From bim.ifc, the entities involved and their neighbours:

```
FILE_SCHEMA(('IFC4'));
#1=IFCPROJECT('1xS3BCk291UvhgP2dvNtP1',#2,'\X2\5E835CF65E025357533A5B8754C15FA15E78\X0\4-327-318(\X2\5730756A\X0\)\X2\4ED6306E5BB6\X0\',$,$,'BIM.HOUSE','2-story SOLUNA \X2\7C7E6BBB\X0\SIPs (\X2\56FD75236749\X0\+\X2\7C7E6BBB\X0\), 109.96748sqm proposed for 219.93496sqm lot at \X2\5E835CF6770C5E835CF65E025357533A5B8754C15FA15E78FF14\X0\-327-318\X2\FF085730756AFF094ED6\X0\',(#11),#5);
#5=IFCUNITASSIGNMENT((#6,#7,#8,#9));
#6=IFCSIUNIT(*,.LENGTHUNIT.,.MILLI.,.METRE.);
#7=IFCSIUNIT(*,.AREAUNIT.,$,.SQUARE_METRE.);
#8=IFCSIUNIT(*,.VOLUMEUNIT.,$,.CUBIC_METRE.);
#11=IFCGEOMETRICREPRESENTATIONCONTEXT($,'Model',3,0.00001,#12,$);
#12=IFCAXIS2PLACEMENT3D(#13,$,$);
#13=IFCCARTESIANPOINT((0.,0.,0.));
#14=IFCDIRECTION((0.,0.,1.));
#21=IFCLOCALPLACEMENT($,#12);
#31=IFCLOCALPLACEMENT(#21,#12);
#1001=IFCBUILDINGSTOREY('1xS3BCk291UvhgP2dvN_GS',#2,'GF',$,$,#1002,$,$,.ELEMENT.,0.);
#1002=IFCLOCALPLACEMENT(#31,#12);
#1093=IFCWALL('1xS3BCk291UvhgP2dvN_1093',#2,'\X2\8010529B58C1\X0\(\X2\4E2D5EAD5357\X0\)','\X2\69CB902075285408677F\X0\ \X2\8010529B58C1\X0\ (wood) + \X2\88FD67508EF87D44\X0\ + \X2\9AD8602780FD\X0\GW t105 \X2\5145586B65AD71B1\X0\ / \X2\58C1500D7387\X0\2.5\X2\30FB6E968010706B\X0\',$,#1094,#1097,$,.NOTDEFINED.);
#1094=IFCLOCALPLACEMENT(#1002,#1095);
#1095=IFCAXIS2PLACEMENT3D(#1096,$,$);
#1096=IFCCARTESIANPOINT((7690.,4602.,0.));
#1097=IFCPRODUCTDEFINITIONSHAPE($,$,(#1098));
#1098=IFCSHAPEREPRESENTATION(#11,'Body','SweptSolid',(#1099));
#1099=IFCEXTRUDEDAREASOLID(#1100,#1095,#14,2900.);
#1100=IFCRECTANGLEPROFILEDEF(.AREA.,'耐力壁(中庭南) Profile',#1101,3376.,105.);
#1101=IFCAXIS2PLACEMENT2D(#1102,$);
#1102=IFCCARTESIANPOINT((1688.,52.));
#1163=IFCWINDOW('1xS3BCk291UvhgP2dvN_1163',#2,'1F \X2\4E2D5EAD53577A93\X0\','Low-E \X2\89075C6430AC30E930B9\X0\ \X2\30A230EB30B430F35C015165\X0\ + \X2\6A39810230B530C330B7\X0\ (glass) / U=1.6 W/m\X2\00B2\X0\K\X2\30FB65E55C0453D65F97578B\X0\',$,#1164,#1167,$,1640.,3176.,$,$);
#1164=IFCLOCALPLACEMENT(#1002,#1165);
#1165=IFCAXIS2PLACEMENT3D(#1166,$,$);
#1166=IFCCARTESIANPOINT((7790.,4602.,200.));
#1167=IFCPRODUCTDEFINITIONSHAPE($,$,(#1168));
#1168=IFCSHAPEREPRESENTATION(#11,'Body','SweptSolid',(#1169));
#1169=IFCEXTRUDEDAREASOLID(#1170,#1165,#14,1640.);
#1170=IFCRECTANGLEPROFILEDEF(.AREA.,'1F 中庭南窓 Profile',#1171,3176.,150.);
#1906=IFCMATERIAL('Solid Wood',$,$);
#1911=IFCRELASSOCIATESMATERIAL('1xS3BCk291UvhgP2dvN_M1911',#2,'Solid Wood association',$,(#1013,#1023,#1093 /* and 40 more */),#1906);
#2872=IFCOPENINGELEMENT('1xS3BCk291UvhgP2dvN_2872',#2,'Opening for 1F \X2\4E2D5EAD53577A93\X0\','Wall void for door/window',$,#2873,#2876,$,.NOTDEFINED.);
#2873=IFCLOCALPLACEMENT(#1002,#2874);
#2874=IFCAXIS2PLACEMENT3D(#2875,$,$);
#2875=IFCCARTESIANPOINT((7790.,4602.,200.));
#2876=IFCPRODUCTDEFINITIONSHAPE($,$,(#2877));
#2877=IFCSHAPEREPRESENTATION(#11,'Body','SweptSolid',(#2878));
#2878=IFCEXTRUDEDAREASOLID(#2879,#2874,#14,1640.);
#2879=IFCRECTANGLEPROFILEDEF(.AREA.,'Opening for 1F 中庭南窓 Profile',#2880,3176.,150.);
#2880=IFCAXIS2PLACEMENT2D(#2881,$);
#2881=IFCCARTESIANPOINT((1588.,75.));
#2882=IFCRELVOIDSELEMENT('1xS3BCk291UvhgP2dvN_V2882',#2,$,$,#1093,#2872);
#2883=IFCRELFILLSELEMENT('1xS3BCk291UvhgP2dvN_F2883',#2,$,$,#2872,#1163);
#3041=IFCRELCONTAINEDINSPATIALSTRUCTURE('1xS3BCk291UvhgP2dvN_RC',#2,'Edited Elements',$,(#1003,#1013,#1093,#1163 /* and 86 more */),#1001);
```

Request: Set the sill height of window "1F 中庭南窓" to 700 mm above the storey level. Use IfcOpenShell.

```python
import numpy as np
import ifcopenshell
import ifcopenshell.api.geometry
import ifcopenshell.geom
import ifcopenshell.util.element
import ifcopenshell.util.placement
import ifcopenshell.util.shape
import ifcopenshell.util.unit

model = ifcopenshell.open("bim.ifc")
unit_scale = ifcopenshell.util.unit.calculate_unit_scale(model)

window = model.by_guid("1xS3BCk291UvhgP2dvN_1163")
opening = window.FillsVoids[0].RelatingOpeningElement
storey = ifcopenshell.util.element.get_container(window, ifc_class="IfcBuildingStorey")
level = ifcopenshell.util.placement.get_local_placement(storey.ObjectPlacement)[2, 3]

# The opening's origin need not be at the sill, so measure its lowest point.
shape = ifcopenshell.geom.create_shape(ifcopenshell.geom.settings(), opening)
bottom = ifcopenshell.util.shape.get_shape_bottom_elevation(shape, shape.geometry) / unit_scale
dz = level + 0.7 / unit_scale - bottom

shift = np.array([0.0, 0.0, dz])
# The window is not placed relative to its opening, so move both.
for product in (opening, window):
    matrix = ifcopenshell.util.placement.get_local_placement(product.ObjectPlacement)
    matrix[:3, 3] += shift
    ifcopenshell.api.geometry.edit_object_placement(model, product=product, matrix=matrix, is_si=False)

print(f"moved by {dz * unit_scale:+.3f} m")

model.write("bim-out.ifc")
```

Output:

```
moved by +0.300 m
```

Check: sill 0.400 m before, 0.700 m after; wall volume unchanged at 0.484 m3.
